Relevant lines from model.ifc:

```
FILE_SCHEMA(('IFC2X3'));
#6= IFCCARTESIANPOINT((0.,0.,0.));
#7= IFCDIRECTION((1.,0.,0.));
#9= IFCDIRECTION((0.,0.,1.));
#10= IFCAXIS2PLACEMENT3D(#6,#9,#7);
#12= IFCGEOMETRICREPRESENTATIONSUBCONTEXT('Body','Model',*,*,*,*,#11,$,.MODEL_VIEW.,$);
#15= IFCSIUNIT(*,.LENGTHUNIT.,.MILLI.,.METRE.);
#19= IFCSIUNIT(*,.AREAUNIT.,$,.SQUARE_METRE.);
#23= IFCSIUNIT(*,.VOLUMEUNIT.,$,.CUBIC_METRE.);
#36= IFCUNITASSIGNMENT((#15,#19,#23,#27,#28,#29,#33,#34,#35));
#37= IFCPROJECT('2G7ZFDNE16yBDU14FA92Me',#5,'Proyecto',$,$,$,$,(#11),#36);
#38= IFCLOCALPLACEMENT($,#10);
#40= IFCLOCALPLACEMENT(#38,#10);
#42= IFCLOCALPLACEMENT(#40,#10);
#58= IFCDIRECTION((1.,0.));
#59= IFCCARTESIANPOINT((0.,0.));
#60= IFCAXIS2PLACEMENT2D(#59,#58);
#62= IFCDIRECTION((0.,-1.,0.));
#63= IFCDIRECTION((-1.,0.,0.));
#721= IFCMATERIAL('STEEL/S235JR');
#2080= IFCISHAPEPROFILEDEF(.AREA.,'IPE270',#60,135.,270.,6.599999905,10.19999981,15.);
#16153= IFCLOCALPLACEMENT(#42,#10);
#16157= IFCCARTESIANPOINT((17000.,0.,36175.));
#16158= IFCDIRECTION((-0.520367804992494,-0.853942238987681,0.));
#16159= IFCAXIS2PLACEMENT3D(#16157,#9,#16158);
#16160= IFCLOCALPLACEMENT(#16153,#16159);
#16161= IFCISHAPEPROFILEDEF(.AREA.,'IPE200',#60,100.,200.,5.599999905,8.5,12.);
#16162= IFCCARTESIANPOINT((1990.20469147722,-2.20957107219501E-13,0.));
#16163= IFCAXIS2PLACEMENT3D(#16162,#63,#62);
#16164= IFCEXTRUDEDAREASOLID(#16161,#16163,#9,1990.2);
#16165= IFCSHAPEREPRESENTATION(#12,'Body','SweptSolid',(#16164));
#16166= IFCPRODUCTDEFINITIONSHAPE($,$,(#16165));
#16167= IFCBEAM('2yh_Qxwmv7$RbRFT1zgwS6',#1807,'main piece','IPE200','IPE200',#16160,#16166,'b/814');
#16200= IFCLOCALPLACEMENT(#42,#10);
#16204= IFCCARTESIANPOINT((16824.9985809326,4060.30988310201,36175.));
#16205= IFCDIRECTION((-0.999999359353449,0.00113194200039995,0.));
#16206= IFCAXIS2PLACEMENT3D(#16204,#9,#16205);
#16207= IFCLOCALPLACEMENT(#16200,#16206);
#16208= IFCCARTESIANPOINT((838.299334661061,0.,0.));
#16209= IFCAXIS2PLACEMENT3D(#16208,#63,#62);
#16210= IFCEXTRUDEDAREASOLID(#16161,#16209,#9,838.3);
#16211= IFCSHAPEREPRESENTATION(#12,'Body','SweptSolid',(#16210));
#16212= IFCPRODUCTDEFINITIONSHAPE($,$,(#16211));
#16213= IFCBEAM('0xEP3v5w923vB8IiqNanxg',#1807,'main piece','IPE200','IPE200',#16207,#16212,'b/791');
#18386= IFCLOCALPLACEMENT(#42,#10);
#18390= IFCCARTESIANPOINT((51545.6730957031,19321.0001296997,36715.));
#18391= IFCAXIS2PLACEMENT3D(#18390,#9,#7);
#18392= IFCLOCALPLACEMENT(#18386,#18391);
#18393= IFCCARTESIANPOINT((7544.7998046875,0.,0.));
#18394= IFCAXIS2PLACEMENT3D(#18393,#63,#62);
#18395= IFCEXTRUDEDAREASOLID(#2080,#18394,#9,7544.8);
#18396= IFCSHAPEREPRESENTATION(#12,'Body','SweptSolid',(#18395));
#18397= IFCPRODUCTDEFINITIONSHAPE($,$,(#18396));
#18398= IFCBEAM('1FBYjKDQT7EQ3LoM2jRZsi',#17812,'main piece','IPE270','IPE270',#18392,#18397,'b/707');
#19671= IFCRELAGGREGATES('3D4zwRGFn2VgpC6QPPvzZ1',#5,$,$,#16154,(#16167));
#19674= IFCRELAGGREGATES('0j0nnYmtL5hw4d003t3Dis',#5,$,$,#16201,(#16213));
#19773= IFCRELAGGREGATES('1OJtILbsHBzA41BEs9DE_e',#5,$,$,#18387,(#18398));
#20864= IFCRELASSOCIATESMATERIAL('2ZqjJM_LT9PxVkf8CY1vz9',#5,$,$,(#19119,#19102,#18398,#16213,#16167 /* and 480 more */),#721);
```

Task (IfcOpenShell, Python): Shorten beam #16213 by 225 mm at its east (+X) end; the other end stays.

```python
import ifcopenshell
import ifcopenshell.util.representation

model = ifcopenshell.open("model.ifc")

member = model.by_guid("0xEP3v5w923vB8IiqNanxg")
change = -225.0

# The extrusion runs towards the end named, so only its depth changes.
body = ifcopenshell.util.representation.get_representation(member, "Model", "Body")
solid = body.Items[0]
old_length = solid.Depth
solid.Depth += change

print(f"length {old_length:g} -> {solid.Depth:g}")

model.write("model-out.ifc")
```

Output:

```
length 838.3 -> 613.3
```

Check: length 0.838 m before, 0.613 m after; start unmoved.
